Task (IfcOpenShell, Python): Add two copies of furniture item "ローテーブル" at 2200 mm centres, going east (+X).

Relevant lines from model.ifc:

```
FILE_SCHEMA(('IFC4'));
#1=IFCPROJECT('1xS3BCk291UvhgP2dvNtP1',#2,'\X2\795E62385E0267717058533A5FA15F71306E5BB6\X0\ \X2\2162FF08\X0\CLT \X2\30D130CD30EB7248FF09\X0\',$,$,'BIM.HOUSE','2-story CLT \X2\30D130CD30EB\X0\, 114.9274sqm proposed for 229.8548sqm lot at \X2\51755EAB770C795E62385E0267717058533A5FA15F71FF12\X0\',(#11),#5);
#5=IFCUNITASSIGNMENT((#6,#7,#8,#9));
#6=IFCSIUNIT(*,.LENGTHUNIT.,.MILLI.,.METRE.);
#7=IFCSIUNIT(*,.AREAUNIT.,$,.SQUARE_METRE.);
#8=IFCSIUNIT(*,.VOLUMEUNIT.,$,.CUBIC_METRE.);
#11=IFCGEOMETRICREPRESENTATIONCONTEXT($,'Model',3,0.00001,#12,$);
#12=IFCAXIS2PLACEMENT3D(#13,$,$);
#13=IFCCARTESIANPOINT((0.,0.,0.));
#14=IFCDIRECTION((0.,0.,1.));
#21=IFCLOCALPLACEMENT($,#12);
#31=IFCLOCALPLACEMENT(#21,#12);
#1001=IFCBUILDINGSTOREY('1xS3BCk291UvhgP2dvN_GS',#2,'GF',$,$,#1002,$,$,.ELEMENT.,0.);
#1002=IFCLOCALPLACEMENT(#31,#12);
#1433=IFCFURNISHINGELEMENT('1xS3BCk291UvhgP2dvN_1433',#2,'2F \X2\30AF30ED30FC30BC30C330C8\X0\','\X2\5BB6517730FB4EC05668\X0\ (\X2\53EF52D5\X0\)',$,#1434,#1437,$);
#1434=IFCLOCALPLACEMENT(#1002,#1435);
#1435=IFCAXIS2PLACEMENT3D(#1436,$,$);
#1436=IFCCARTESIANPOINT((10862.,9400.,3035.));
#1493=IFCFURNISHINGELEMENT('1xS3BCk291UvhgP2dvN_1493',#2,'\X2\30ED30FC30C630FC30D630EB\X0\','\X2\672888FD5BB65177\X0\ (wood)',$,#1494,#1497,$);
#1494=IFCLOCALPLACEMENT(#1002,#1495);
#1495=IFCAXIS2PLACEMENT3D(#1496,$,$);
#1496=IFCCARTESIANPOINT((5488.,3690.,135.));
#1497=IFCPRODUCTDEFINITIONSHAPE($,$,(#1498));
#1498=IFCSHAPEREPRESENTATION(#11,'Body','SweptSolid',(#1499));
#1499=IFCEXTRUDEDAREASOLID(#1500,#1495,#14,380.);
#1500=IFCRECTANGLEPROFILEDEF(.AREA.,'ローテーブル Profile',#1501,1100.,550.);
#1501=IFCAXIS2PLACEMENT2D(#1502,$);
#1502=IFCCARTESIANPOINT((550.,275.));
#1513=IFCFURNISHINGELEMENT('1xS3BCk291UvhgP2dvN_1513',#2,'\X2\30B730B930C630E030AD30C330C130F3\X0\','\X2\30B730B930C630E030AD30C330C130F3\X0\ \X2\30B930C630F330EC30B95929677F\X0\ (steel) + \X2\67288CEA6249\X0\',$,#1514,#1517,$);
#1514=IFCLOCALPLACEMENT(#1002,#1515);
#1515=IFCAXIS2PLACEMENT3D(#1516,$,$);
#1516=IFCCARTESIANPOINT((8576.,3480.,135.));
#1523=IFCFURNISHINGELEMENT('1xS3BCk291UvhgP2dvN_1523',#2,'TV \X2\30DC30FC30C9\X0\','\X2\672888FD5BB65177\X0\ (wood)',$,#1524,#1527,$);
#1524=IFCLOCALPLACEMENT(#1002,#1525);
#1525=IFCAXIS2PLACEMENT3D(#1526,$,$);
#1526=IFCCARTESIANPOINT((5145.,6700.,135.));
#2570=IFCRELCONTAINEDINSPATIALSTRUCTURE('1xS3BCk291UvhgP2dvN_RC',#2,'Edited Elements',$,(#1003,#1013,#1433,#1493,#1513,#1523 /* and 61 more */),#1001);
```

```python
import numpy as np
import ifcopenshell
import ifcopenshell.api.geometry
import ifcopenshell.api.root
import ifcopenshell.util.element
import ifcopenshell.util.placement
import ifcopenshell.util.unit

model = ifcopenshell.open("model.ifc")
unit_scale = ifcopenshell.util.unit.calculate_unit_scale(model)


def reuse_history(source, copy):
    """copy_class also copies each property set's owner history, people and application; keep the originals."""
    for rel in copy.IsDefinedBy:
        if rel.is_a("IfcRelDefinesByProperties") and (history := rel.RelatingPropertyDefinition.OwnerHistory):
            rel.RelatingPropertyDefinition.OwnerHistory = source.OwnerHistory
            ifcopenshell.util.element.remove_deep2(model, history)


source = model.by_guid("1xS3BCk291UvhgP2dvN_1493")
base = ifcopenshell.util.placement.get_local_placement(source.ObjectPlacement)
step = np.array([1.0, 0.0, 0.0]) * 2.2 / unit_scale

for i in range(1, 3):
    copy = ifcopenshell.api.root.copy_class(model, product=source)
    copy.Representation = ifcopenshell.util.element.copy_deep(
        model, source.Representation, exclude=["IfcGeometricRepresentationContext", "IfcRepresentationMap"]
    )
    reuse_history(source, copy)
    matrix = base.copy()
    matrix[:3, 3] += i * step
    print("added at", matrix[:3, 3].round(3) + 0.0)
    ifcopenshell.api.geometry.edit_object_placement(model, product=copy, matrix=matrix, is_si=False)

model.write("model-out.ifc")
```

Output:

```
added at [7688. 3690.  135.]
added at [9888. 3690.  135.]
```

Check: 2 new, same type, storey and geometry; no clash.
